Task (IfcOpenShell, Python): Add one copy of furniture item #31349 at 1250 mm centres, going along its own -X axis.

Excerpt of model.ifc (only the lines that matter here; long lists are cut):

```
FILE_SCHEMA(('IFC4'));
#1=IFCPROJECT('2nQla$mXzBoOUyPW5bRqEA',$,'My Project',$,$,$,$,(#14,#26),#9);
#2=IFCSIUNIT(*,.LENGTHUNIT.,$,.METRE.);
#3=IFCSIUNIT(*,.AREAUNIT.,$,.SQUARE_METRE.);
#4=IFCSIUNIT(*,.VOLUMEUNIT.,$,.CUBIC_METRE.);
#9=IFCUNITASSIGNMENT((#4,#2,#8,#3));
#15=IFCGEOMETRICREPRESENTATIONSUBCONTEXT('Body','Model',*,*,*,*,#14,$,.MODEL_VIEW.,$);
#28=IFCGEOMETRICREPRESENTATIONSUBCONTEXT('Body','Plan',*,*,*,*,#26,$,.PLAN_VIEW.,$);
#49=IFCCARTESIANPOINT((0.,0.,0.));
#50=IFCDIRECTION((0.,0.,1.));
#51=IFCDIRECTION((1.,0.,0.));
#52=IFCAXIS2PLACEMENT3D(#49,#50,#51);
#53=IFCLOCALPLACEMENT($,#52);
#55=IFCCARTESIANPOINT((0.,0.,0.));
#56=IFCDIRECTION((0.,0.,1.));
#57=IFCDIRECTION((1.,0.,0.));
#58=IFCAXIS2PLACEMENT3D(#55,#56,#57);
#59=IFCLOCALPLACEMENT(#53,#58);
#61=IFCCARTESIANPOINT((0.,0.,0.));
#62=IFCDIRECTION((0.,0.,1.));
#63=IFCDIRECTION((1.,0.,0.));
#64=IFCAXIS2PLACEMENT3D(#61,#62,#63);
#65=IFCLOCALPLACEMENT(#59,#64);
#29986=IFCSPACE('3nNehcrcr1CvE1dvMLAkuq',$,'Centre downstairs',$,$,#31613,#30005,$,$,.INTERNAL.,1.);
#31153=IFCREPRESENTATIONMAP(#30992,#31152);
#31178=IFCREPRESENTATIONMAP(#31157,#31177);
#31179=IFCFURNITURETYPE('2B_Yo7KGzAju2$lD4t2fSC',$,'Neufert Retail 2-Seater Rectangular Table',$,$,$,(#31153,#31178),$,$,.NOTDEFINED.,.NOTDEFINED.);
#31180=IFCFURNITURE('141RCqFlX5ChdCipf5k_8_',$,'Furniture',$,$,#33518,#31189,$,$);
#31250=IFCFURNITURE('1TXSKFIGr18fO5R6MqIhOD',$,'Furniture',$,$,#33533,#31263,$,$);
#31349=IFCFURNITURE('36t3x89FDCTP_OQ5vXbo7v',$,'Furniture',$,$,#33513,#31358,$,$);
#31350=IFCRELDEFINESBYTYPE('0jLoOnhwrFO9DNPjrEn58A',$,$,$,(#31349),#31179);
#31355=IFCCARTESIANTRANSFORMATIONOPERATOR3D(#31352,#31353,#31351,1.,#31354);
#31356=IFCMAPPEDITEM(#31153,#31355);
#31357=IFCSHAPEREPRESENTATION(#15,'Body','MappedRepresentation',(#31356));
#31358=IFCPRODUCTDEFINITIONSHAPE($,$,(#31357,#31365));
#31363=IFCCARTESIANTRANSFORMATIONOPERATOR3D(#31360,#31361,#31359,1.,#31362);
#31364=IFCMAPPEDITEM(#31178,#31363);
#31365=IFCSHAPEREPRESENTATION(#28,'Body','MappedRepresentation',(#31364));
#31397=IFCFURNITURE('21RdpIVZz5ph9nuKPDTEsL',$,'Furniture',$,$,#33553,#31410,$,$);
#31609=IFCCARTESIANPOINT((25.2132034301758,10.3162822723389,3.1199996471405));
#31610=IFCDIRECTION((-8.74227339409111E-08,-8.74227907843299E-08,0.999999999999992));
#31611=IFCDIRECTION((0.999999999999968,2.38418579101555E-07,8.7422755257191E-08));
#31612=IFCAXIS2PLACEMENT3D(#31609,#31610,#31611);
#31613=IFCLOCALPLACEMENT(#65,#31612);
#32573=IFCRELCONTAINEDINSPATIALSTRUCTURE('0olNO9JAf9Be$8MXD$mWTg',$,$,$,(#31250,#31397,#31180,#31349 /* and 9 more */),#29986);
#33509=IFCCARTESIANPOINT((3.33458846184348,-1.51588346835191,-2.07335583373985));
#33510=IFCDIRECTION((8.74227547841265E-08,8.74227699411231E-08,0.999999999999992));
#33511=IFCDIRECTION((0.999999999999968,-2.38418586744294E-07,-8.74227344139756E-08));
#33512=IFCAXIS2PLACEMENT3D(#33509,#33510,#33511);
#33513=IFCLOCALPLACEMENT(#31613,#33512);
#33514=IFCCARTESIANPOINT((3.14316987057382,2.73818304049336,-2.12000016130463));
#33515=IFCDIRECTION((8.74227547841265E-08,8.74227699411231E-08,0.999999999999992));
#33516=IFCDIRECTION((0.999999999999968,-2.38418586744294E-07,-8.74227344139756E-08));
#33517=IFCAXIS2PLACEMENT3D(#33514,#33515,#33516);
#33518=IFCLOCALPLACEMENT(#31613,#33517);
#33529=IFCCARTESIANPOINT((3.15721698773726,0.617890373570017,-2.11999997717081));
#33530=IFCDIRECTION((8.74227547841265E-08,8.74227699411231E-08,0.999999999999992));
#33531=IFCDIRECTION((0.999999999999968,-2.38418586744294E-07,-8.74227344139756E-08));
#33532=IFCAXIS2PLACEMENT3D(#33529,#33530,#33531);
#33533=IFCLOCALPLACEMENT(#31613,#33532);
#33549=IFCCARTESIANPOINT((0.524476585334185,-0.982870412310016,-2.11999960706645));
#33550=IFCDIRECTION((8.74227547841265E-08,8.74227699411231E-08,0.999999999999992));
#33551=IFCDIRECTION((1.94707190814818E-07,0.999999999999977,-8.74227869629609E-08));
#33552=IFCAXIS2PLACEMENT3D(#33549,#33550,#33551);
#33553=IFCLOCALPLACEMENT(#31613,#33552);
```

```python
import ifcopenshell
import ifcopenshell.api.geometry
import ifcopenshell.api.root
import ifcopenshell.util.element
import ifcopenshell.util.placement

model = ifcopenshell.open("model.ifc")

source = model.by_guid("36t3x89FDCTP_OQ5vXbo7v")
base = ifcopenshell.util.placement.get_local_placement(source.ObjectPlacement)
step = -base[:3, 0] * 1.25

for i in range(1, 2):
    copy = ifcopenshell.api.root.copy_class(model, product=source)
    copy.Representation = ifcopenshell.util.element.copy_deep(
        model, source.Representation, exclude=["IfcGeometricRepresentationContext", "IfcRepresentationMap"]
    )
    matrix = base.copy()
    matrix[:3, 3] += i * step
    print("added at", matrix[:3, 3].round(3) + 0.0)
    ifcopenshell.api.geometry.edit_object_placement(model, product=copy, matrix=matrix, is_si=False)

model.write("model_edited.ifc")
```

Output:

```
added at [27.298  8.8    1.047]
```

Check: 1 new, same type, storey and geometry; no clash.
